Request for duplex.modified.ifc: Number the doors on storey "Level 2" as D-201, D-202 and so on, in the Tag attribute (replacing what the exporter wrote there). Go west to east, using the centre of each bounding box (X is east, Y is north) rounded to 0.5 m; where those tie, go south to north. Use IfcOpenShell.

First a look at what the model holds.

```python
import ifcopenshell
import ifcopenshell.util.element
import ifcopenshell.util.placement

model = ifcopenshell.open("duplex.modified.ifc")
print(model.schema)
storey = next(s for s in model.by_type("IfcBuildingStorey") if s.Name == "Level 2")
doors = [e for e in ifcopenshell.util.element.get_decomposition(storey) if e.is_a("IfcDoor")]
for e in sorted(doors, key=lambda e: e.id()):
    origin = ifcopenshell.util.placement.get_local_placement(e.ObjectPlacement)[:3, 3]
    print(e.id(), e.Tag, e.Name, origin.round(2) + 0.0, sep=" | ")
```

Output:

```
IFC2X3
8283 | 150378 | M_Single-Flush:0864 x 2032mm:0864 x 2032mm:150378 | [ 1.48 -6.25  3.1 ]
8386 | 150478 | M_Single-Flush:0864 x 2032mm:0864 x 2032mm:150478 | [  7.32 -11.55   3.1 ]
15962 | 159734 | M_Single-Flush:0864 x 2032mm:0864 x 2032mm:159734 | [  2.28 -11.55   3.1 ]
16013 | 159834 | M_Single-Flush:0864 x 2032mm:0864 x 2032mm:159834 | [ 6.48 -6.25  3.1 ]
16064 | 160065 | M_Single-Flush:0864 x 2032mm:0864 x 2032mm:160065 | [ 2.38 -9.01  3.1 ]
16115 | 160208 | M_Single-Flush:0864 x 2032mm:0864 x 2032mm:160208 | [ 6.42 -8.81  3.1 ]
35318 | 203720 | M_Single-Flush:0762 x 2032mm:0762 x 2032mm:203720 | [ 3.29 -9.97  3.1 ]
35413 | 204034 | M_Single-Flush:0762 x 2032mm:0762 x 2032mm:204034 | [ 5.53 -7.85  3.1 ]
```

```python
import ifcopenshell
import ifcopenshell.geom
import ifcopenshell.util.element
import ifcopenshell.util.shape

model = ifcopenshell.open("duplex.modified.ifc")
settings = ifcopenshell.geom.settings()
settings.set("use-world-coords", True)


def centre(element):
    shape = ifcopenshell.geom.create_shape(settings, element)
    return ifcopenshell.util.shape.get_bbox_centroid(shape.geometry)


storey = next(s for s in model.by_type("IfcBuildingStorey") if s.Name == "Level 2")
doors = [e for e in ifcopenshell.util.element.get_decomposition(storey) if e.is_a("IfcDoor")]

# Insertion points can sit at a corner or the storey origin, so sort by the geometry (in metres).
centres = {e: centre(e) for e in doors}
doors.sort(key=lambda e: (round(centres[e][0] / 0.5), centres[e][1]))

for i, e in enumerate(doors, start=1):
    number = f"D-2{i:02d}"
    e.Tag = number
    print(e.id(), number)

model.write("duplex.modified_rev.ifc")
```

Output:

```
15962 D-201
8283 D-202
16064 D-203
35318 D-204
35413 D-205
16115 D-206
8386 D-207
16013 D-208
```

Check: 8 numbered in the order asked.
